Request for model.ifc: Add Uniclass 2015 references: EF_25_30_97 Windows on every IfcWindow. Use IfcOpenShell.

First a look at what the model holds.

```python
import ifcopenshell

model = ifcopenshell.open("model.ifc")
print(model.schema)
print("classifications:", [c.Name for c in model.by_type("IfcClassification")])
for ifc_class in ("IfcDoor", "IfcRoof", "IfcStair", "IfcWall", "IfcWindow"):
    print(ifc_class, len(model.by_type(ifc_class)))
```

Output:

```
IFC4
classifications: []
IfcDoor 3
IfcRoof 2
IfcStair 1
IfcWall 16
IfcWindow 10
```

```python
import ifcopenshell
import ifcopenshell.api.classification

model = ifcopenshell.open("model.ifc")

system = ifcopenshell.api.classification.add_classification(model, classification="Uniclass 2015")

codes = {
    "IfcWindow": ("EF_25_30_97", "Windows"),
}
for ifc_class, (code, name) in codes.items():
    products = model.by_type(ifc_class)
    ifcopenshell.api.classification.add_reference(
        model, products=products, classification=system, identification=code, name=name
    )
    print(code, len(products))

model.write("model-out.ifc")
```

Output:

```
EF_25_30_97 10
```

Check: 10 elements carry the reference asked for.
